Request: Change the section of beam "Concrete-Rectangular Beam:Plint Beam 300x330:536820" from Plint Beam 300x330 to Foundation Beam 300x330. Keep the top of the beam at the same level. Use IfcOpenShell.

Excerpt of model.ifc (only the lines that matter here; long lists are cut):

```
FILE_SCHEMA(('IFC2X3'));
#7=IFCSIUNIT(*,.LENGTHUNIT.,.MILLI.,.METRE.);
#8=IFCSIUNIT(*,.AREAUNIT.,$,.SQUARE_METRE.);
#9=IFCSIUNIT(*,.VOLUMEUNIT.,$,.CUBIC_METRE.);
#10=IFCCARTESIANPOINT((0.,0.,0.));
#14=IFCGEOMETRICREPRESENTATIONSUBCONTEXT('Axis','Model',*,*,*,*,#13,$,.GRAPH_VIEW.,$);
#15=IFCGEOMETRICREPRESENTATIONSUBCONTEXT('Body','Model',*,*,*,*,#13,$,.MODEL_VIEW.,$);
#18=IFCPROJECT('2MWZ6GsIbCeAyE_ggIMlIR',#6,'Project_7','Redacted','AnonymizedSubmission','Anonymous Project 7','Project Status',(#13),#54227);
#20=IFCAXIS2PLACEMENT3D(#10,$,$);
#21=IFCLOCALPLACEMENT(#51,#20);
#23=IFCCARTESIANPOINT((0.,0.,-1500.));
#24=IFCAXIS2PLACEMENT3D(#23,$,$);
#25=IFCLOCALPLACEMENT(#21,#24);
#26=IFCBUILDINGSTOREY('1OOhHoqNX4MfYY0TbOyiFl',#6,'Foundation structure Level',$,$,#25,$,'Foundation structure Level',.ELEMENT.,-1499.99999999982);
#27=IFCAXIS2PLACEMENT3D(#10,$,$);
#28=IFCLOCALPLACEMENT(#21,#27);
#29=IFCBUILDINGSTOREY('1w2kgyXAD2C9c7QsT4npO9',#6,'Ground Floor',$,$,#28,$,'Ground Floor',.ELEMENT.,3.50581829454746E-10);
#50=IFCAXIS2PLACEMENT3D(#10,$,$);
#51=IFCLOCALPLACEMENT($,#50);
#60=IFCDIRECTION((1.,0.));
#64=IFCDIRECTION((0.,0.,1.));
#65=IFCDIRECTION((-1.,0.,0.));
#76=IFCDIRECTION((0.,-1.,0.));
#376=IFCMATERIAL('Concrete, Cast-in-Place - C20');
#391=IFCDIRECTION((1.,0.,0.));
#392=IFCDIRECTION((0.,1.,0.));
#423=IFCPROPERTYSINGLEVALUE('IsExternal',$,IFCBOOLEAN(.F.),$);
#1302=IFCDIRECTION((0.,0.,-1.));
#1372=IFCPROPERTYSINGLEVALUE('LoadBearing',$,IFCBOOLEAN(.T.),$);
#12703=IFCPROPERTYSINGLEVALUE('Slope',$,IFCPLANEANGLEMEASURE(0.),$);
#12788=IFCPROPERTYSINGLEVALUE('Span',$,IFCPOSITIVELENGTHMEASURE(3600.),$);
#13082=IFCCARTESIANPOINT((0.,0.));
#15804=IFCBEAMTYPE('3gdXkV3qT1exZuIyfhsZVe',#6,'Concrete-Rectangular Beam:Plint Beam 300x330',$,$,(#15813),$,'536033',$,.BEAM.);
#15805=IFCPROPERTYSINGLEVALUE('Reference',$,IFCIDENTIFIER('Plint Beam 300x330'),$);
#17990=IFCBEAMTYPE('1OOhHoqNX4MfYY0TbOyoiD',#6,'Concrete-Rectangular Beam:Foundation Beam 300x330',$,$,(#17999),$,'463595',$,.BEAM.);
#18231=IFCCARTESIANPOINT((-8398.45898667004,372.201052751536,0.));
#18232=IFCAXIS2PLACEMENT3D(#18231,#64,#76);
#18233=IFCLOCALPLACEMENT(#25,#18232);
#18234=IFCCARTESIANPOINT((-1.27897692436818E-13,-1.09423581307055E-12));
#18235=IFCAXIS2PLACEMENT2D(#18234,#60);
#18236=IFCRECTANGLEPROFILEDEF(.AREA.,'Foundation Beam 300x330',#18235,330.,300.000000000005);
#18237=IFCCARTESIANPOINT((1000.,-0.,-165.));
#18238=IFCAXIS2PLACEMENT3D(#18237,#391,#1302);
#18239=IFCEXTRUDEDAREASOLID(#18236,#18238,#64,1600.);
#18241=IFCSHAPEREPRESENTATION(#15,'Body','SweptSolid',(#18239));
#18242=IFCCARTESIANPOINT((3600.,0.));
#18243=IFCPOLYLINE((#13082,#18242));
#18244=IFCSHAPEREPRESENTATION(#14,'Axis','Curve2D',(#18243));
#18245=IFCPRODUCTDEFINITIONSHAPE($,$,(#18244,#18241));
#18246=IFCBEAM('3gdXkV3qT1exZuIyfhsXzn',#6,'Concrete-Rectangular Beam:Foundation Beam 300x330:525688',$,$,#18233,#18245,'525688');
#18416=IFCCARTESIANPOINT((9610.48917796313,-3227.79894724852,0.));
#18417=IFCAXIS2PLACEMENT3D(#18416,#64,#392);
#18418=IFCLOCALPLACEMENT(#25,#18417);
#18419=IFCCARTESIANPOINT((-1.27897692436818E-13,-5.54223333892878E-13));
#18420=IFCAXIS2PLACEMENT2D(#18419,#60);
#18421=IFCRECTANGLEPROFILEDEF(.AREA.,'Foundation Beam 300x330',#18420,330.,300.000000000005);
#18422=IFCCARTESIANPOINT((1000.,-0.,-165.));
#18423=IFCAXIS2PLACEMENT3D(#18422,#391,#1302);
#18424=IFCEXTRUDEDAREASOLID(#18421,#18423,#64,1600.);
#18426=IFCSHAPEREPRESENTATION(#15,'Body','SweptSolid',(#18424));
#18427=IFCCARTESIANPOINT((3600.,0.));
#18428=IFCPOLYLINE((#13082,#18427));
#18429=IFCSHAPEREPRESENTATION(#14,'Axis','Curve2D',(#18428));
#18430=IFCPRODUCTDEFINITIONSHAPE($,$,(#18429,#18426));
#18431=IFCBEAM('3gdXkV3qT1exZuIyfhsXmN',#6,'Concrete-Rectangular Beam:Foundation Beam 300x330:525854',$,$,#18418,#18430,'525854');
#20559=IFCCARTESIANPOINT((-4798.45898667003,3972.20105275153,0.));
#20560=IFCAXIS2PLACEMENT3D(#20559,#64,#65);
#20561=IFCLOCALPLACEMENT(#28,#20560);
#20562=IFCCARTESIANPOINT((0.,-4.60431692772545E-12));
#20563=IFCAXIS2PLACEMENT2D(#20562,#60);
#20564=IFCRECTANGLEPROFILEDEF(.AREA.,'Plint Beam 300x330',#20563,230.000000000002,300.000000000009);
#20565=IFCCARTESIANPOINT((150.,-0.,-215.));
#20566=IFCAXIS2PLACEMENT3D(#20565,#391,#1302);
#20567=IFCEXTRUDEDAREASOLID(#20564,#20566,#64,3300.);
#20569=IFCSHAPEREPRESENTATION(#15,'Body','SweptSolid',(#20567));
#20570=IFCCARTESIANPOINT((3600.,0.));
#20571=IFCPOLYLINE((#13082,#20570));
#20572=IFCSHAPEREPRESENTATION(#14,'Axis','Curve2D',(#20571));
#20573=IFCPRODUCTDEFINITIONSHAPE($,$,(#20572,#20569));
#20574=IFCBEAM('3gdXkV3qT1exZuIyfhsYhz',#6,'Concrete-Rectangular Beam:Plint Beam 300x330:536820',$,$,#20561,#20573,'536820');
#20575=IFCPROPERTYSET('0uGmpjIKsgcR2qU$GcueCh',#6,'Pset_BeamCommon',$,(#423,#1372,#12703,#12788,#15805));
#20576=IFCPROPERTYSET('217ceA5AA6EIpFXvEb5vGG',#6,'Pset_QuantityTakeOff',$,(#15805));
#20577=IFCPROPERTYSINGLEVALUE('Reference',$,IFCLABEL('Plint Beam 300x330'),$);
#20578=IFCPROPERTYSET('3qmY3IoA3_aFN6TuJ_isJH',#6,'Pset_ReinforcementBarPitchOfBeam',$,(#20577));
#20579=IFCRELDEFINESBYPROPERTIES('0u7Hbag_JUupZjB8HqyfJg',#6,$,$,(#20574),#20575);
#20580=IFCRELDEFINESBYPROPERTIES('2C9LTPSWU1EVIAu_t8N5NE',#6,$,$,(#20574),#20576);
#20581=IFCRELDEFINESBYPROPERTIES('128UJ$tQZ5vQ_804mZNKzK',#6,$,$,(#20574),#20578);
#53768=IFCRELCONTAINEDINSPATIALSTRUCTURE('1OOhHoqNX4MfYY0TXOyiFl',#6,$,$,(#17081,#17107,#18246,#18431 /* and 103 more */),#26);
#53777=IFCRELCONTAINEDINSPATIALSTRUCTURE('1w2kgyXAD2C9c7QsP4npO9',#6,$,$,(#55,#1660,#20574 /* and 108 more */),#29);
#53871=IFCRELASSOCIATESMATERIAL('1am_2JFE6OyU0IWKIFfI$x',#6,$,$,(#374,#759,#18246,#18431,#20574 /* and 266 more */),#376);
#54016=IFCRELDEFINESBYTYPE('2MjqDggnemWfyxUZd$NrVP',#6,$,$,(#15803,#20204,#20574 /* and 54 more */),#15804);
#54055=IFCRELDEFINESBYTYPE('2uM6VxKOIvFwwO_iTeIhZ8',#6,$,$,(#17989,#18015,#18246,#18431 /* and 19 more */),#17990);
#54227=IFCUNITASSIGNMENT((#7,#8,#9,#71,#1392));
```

```python
import ifcopenshell
import ifcopenshell.api.pset
import ifcopenshell.api.type
import ifcopenshell.util.element
import ifcopenshell.util.representation

model = ifcopenshell.open("model.ifc")

member = model.by_id(20574)
source = next(p for p in model.by_type("IfcRectangleProfileDef") if p.ProfileName == "Foundation Beam 300x330")

body = ifcopenshell.util.representation.get_representation(member, "Model", "Body")
solid = body.Items[0]
old_profile = solid.SweptArea

# Copy the section's sizes but keep this member's own profile position.
profile = ifcopenshell.util.element.copy(model, source)
# Profiles are centred, so shift by half the change in depth to hold the top.
shift = (old_profile.XDim - profile.XDim) / 2
x, y = old_profile.Position.Location.Coordinates
up = (-1.0, 0.0)  # upwards, in the solid's own plane
location = model.createIfcCartesianPoint((x + up[0] * shift, y + up[1] * shift))
profile.Position = model.createIfcAxis2Placement2D(location, old_profile.Position.RefDirection)
solid.SweptArea = profile
if not model.get_total_inverses(old_profile):
    ifcopenshell.util.element.remove_deep2(model, old_profile)

new_type = model.by_guid("1OOhHoqNX4MfYY0TbOyoiD")
ifcopenshell.api.type.assign_type(
    model, related_objects=[member], relating_type=new_type, should_map_representations=False
)
member.Name = member.Name.replace("Plint Beam 300x330", "Foundation Beam 300x330")
pset = model.by_id(ifcopenshell.util.element.get_pset(member, "Pset_BeamCommon", should_inherit=False)["id"])
ifcopenshell.api.pset.edit_pset(model, pset=pset, properties={"Reference": "Foundation Beam 300x330"})
pset = model.by_id(ifcopenshell.util.element.get_pset(member, "Pset_QuantityTakeOff", should_inherit=False)["id"])
ifcopenshell.api.pset.edit_pset(model, pset=pset, properties={"Reference": "Foundation Beam 300x330"})
pset = model.by_id(ifcopenshell.util.element.get_pset(member, "Pset_ReinforcementBarPitchOfBeam", should_inherit=False)["id"])
ifcopenshell.api.pset.edit_pset(model, pset=pset, properties={"Reference": "Foundation Beam 300x330"})

print(solid.SweptArea)

model.write("model_v2.ifc")
```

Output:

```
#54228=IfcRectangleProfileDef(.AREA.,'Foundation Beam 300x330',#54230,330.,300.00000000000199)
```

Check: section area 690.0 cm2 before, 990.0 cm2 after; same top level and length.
